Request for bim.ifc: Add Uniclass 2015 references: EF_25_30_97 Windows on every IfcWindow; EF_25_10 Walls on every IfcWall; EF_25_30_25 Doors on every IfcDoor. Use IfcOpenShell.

First a look at what the model holds.

```python
import ifcopenshell

model = ifcopenshell.open("bim.ifc")
print(model.schema)
print("classifications:", [c.Name for c in model.by_type("IfcClassification")])
for ifc_class in ("IfcDoor", "IfcRoof", "IfcStair", "IfcWall", "IfcWindow"):
    print(ifc_class, len(model.by_type(ifc_class)))
```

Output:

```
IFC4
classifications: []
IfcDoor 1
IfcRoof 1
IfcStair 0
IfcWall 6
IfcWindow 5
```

```python
import ifcopenshell
import ifcopenshell.api.classification

model = ifcopenshell.open("bim.ifc")

system = ifcopenshell.api.classification.add_classification(model, classification="Uniclass 2015")

codes = {
    "IfcWindow": ("EF_25_30_97", "Windows"),
    "IfcWall": ("EF_25_10", "Walls"),
    "IfcDoor": ("EF_25_30_25", "Doors"),
}
for ifc_class, (code, name) in codes.items():
    products = model.by_type(ifc_class)
    ifcopenshell.api.classification.add_reference(
        model, products=products, classification=system, identification=code, name=name
    )
    print(code, len(products))

model.write("bim-out.ifc")
```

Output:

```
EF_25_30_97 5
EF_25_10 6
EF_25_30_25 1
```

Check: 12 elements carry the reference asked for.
